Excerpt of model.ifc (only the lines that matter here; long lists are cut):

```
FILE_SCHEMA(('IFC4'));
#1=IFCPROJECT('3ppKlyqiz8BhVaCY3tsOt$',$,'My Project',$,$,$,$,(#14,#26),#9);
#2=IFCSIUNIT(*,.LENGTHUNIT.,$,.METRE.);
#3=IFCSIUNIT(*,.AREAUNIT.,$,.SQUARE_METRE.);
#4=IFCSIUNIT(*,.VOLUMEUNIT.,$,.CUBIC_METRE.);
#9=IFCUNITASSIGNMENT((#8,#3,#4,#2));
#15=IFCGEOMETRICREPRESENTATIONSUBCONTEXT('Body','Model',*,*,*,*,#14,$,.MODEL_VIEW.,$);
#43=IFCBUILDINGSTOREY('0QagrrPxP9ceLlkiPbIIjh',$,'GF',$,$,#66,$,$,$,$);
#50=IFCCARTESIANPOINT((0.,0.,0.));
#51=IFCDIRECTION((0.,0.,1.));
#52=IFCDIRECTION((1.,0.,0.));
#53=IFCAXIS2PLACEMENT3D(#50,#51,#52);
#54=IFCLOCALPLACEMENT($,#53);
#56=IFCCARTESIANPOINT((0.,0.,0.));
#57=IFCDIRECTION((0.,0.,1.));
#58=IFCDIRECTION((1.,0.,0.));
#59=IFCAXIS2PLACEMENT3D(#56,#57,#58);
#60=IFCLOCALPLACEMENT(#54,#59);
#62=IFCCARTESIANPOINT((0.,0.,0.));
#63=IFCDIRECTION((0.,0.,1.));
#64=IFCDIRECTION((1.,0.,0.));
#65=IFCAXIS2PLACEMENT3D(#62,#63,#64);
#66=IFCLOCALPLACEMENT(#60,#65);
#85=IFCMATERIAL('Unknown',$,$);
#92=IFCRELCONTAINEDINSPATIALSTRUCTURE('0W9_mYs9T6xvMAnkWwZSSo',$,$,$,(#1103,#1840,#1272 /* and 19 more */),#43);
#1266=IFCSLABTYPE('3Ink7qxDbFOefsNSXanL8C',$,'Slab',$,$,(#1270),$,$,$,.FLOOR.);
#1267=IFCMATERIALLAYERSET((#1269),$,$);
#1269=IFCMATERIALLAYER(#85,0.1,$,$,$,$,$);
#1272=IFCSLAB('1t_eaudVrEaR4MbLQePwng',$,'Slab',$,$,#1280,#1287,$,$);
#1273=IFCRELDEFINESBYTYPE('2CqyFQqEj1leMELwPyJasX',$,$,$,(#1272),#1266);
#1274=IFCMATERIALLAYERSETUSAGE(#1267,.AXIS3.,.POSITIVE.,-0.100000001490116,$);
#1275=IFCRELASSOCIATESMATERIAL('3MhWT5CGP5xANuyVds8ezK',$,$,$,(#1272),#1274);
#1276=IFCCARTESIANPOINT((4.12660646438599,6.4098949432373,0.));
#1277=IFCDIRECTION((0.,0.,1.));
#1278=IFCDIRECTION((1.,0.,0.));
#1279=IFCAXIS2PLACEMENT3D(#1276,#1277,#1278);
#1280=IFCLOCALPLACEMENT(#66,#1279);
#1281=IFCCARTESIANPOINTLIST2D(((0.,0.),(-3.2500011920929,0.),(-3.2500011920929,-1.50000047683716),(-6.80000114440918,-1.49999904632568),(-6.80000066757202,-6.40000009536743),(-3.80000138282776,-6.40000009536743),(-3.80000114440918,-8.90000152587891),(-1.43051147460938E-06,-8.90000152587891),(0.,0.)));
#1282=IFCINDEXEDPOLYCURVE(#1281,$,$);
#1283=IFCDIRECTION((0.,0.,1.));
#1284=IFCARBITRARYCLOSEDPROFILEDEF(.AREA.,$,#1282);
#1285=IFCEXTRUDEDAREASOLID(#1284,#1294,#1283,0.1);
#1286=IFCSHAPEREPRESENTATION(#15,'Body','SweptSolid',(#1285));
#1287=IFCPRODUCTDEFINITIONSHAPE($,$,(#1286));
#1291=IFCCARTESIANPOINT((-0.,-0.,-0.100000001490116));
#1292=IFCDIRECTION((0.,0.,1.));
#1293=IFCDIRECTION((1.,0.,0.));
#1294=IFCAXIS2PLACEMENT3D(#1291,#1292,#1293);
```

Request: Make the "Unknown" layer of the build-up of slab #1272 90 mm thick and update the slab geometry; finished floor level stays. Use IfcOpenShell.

```python
import ifcopenshell
import ifcopenshell.util.element
import ifcopenshell.util.representation
import ifcopenshell.util.unit

model = ifcopenshell.open("model.ifc")
unit_scale = ifcopenshell.util.unit.calculate_unit_scale(model)

layer_set = model.by_id(1267)
layer = next(l for l in layer_set.MaterialLayers if l.Material and l.Material.Name == "Unknown")
change = 0.09 / unit_scale - layer.LayerThickness
layer.LayerThickness += change

# Geometry does not follow the layer set by itself.
slabs = [e for e in ifcopenshell.util.element.get_elements_by_material(model, layer_set) if e.is_a("IfcSlab")]
for slab in sorted(slabs, key=lambda e: e.id()):
    body = ifcopenshell.util.representation.get_representation(slab, "Model", "Body")
    solid = body.Items[0]
    old_depth = solid.Depth
    solid.Depth += change
    # Extruded upwards: lower the start of the extrusion so the top stays.
    x, y, z = solid.Position.Location.Coordinates
    solid.Position.Location = model.createIfcCartesianPoint((x, y, z - change))
    print(slab.id(), f"{old_depth:g} -> {solid.Depth:g}")

# The layers are counted up from the underside, which has moved.
for usage in {ifcopenshell.util.element.get_material(slab) for slab in slabs}:
    usage.OffsetFromReferenceLine -= change

model.write("model_v2.ifc")
```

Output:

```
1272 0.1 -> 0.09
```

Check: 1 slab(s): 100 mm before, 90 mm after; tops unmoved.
